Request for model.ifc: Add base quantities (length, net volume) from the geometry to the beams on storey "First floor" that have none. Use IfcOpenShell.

First a look at what the model holds.

```python
import ifcopenshell
import ifcopenshell.util.element
import ifcopenshell.util.unit

model = ifcopenshell.open("model.ifc")
print(model.schema)
for unit_type in ("LENGTHUNIT", "AREAUNIT", "VOLUMEUNIT"):
    print(unit_type, ifcopenshell.util.unit.calculate_unit_scale(model, unit_type))
storey = next(s for s in model.by_type("IfcBuildingStorey") if s.Name == "First floor")
beams = [e for e in ifcopenshell.util.element.get_decomposition(storey) if e.is_a("IfcBeam")]
for e in sorted(beams, key=lambda e: e.id()):
    print(e.id(), e.is_a(), e.Name, list(ifcopenshell.util.element.get_psets(e, qtos_only=True)), sep=" | ")
```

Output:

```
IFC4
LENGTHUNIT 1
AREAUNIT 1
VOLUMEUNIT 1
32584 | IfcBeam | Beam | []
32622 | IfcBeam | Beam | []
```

```python
import ifcopenshell
import ifcopenshell.api.pset
import ifcopenshell.geom
import ifcopenshell.util.element
import ifcopenshell.util.shape
import ifcopenshell.util.unit

model = ifcopenshell.open("model.ifc")
unit_scale = ifcopenshell.util.unit.calculate_unit_scale(model)
volume_scale = ifcopenshell.util.unit.calculate_unit_scale(model, "VOLUMEUNIT")
settings = ifcopenshell.geom.settings()

storey = next(s for s in model.by_type("IfcBuildingStorey") if s.Name == "First floor")
beams = [e for e in ifcopenshell.util.element.get_decomposition(storey) if e.is_a("IfcBeam")]

for e in sorted(beams, key=lambda e: e.id()):
    if ifcopenshell.util.element.get_psets(e, qtos_only=True, should_inherit=False):
        continue
    # Geometry comes back in metres, in the element's own axes.
    shape = ifcopenshell.geom.create_shape(settings, e)
    values = {
        "Length": ifcopenshell.util.shape.get_max_xyz(shape.geometry) / unit_scale,
        "NetVolume": ifcopenshell.util.shape.get_volume(shape.geometry) / volume_scale,
    }
    qto = ifcopenshell.api.pset.add_qto(model, product=e, name="Qto_BeamBaseQuantities")
    ifcopenshell.api.pset.edit_qto(model, qto=qto, properties=values)
    print(e.id(), {k: round(v, 3) for k, v in values.items()})

model.write("model_updated.ifc")
```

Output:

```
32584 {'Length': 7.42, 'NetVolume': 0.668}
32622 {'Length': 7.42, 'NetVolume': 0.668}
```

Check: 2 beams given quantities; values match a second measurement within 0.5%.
